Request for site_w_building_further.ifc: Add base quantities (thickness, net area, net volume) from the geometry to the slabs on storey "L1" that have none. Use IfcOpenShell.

First a look at what the model holds.

```python
import ifcopenshell
import ifcopenshell.util.element
import ifcopenshell.util.unit

model = ifcopenshell.open("site_w_building_further.ifc")
print(model.schema)
for unit_type in ("LENGTHUNIT", "AREAUNIT", "VOLUMEUNIT"):
    print(unit_type, ifcopenshell.util.unit.calculate_unit_scale(model, unit_type))
storey = next(s for s in model.by_type("IfcBuildingStorey") if s.Name == "L1")
slabs = [e for e in ifcopenshell.util.element.get_decomposition(storey) if e.is_a("IfcSlab")]
for e in sorted(slabs, key=lambda e: e.id()):
    print(e.id(), e.is_a(), e.Name, list(ifcopenshell.util.element.get_psets(e, qtos_only=True)), sep=" | ")
```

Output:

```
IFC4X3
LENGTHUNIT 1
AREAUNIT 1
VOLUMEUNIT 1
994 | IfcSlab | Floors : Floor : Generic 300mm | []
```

```python
import ifcopenshell
import ifcopenshell.api.pset
import ifcopenshell.geom
import ifcopenshell.util.element
import ifcopenshell.util.shape
import ifcopenshell.util.unit

model = ifcopenshell.open("site_w_building_further.ifc")
unit_scale = ifcopenshell.util.unit.calculate_unit_scale(model)
area_scale = ifcopenshell.util.unit.calculate_unit_scale(model, "AREAUNIT")
volume_scale = ifcopenshell.util.unit.calculate_unit_scale(model, "VOLUMEUNIT")
settings = ifcopenshell.geom.settings()

storey = next(s for s in model.by_type("IfcBuildingStorey") if s.Name == "L1")
slabs = [e for e in ifcopenshell.util.element.get_decomposition(storey) if e.is_a("IfcSlab")]

for e in sorted(slabs, key=lambda e: e.id()):
    if ifcopenshell.util.element.get_psets(e, qtos_only=True, should_inherit=False):
        continue
    # Geometry comes back in metres, in the element's own axes.
    shape = ifcopenshell.geom.create_shape(settings, e)
    values = {
        "Width": ifcopenshell.util.shape.get_z(shape.geometry) / unit_scale,
        "NetArea": ifcopenshell.util.shape.get_footprint_area(shape.geometry) / area_scale,
        "NetVolume": ifcopenshell.util.shape.get_volume(shape.geometry) / volume_scale,
    }
    qto = ifcopenshell.api.pset.add_qto(model, product=e, name="Qto_SlabBaseQuantities")
    ifcopenshell.api.pset.edit_qto(model, qto=qto, properties=values)
    print(e.id(), {k: round(v, 3) for k, v in values.items()})

model.write("site_w_building_further_v2.ifc")
```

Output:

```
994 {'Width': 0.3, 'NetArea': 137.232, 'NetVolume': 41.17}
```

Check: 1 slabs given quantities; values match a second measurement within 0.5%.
